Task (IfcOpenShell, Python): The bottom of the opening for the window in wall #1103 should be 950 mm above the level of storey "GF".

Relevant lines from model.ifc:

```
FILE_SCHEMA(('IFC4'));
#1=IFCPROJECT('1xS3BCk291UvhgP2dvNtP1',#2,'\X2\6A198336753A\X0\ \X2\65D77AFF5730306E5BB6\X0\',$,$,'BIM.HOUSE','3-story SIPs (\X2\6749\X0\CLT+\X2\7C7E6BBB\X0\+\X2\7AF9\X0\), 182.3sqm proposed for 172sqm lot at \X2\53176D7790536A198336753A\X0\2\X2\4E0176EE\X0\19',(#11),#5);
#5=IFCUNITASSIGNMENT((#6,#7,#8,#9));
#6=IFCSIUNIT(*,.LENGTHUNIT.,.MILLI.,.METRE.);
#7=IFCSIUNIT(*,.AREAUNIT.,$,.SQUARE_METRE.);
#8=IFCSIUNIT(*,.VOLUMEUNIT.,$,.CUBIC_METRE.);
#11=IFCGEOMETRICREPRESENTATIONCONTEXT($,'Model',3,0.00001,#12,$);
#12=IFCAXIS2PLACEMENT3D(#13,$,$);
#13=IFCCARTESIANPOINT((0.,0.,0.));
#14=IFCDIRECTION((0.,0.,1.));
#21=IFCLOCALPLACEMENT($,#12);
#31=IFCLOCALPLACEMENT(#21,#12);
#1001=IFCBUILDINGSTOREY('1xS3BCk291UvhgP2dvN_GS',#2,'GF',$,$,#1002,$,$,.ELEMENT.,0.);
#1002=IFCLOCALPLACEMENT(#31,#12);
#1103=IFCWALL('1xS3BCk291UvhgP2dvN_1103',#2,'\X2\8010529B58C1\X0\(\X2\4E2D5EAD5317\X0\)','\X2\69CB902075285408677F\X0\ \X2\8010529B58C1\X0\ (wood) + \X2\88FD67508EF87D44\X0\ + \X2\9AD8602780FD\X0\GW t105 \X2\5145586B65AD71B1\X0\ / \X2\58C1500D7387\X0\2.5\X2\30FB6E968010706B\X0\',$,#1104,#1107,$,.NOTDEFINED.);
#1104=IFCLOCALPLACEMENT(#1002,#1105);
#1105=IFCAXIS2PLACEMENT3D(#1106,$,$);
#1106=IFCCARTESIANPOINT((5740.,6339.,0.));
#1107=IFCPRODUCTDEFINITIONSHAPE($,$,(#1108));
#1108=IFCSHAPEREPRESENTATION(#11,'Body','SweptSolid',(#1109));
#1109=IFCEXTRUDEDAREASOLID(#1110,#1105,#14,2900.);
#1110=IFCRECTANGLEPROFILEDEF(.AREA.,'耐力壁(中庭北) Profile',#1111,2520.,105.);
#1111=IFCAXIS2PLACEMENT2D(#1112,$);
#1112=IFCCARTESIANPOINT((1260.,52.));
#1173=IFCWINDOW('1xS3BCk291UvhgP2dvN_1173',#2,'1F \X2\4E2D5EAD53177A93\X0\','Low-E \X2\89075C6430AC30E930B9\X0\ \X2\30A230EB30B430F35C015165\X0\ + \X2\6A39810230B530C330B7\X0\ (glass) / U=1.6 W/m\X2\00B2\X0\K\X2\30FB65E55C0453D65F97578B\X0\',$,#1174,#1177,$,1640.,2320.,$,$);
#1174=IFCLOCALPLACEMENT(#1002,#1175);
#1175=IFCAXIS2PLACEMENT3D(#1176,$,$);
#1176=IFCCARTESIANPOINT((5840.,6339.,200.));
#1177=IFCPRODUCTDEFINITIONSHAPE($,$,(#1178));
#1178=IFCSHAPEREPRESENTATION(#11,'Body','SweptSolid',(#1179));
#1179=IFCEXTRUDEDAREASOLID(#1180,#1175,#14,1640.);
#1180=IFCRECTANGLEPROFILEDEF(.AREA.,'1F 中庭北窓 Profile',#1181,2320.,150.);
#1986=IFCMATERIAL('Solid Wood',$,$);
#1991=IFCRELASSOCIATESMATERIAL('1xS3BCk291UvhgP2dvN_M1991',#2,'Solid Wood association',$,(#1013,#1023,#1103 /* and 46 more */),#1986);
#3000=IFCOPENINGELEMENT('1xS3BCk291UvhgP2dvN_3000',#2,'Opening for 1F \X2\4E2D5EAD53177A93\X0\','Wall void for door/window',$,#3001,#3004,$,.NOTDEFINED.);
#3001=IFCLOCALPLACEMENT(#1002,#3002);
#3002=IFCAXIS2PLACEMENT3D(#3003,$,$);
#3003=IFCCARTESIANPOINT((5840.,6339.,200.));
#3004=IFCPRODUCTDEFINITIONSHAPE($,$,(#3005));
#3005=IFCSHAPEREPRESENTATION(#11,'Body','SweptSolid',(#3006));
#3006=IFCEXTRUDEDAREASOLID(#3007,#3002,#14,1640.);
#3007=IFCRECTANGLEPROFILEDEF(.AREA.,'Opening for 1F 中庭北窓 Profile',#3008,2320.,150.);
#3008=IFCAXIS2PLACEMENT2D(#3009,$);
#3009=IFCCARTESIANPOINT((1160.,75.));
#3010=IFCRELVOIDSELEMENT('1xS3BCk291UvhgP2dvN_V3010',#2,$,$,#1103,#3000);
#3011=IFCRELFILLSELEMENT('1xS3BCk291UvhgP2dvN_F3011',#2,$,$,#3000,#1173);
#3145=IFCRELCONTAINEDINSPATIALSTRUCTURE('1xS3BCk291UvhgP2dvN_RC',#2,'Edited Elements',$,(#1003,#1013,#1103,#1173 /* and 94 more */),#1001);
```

```python
import numpy as np
import ifcopenshell
import ifcopenshell.api.geometry
import ifcopenshell.geom
import ifcopenshell.util.element
import ifcopenshell.util.placement
import ifcopenshell.util.shape
import ifcopenshell.util.unit

model = ifcopenshell.open("model.ifc")
unit_scale = ifcopenshell.util.unit.calculate_unit_scale(model)

window = model.by_id(1173)
opening = window.FillsVoids[0].RelatingOpeningElement
storey = ifcopenshell.util.element.get_container(window, ifc_class="IfcBuildingStorey")
level = ifcopenshell.util.placement.get_local_placement(storey.ObjectPlacement)[2, 3]

# The opening's origin need not be at the sill, so measure its lowest point.
shape = ifcopenshell.geom.create_shape(ifcopenshell.geom.settings(), opening)
bottom = ifcopenshell.util.shape.get_shape_bottom_elevation(shape, shape.geometry) / unit_scale
dz = level + 0.95 / unit_scale - bottom

shift = np.array([0.0, 0.0, dz])
# The window is not placed relative to its opening, so move both.
for product in (opening, window):
    matrix = ifcopenshell.util.placement.get_local_placement(product.ObjectPlacement)
    matrix[:3, 3] += shift
    ifcopenshell.api.geometry.edit_object_placement(model, product=product, matrix=matrix, is_si=False)

print(f"moved by {dz * unit_scale:+.3f} m")

model.write("model_rev.ifc")
```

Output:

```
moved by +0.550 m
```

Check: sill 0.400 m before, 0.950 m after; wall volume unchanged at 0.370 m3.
